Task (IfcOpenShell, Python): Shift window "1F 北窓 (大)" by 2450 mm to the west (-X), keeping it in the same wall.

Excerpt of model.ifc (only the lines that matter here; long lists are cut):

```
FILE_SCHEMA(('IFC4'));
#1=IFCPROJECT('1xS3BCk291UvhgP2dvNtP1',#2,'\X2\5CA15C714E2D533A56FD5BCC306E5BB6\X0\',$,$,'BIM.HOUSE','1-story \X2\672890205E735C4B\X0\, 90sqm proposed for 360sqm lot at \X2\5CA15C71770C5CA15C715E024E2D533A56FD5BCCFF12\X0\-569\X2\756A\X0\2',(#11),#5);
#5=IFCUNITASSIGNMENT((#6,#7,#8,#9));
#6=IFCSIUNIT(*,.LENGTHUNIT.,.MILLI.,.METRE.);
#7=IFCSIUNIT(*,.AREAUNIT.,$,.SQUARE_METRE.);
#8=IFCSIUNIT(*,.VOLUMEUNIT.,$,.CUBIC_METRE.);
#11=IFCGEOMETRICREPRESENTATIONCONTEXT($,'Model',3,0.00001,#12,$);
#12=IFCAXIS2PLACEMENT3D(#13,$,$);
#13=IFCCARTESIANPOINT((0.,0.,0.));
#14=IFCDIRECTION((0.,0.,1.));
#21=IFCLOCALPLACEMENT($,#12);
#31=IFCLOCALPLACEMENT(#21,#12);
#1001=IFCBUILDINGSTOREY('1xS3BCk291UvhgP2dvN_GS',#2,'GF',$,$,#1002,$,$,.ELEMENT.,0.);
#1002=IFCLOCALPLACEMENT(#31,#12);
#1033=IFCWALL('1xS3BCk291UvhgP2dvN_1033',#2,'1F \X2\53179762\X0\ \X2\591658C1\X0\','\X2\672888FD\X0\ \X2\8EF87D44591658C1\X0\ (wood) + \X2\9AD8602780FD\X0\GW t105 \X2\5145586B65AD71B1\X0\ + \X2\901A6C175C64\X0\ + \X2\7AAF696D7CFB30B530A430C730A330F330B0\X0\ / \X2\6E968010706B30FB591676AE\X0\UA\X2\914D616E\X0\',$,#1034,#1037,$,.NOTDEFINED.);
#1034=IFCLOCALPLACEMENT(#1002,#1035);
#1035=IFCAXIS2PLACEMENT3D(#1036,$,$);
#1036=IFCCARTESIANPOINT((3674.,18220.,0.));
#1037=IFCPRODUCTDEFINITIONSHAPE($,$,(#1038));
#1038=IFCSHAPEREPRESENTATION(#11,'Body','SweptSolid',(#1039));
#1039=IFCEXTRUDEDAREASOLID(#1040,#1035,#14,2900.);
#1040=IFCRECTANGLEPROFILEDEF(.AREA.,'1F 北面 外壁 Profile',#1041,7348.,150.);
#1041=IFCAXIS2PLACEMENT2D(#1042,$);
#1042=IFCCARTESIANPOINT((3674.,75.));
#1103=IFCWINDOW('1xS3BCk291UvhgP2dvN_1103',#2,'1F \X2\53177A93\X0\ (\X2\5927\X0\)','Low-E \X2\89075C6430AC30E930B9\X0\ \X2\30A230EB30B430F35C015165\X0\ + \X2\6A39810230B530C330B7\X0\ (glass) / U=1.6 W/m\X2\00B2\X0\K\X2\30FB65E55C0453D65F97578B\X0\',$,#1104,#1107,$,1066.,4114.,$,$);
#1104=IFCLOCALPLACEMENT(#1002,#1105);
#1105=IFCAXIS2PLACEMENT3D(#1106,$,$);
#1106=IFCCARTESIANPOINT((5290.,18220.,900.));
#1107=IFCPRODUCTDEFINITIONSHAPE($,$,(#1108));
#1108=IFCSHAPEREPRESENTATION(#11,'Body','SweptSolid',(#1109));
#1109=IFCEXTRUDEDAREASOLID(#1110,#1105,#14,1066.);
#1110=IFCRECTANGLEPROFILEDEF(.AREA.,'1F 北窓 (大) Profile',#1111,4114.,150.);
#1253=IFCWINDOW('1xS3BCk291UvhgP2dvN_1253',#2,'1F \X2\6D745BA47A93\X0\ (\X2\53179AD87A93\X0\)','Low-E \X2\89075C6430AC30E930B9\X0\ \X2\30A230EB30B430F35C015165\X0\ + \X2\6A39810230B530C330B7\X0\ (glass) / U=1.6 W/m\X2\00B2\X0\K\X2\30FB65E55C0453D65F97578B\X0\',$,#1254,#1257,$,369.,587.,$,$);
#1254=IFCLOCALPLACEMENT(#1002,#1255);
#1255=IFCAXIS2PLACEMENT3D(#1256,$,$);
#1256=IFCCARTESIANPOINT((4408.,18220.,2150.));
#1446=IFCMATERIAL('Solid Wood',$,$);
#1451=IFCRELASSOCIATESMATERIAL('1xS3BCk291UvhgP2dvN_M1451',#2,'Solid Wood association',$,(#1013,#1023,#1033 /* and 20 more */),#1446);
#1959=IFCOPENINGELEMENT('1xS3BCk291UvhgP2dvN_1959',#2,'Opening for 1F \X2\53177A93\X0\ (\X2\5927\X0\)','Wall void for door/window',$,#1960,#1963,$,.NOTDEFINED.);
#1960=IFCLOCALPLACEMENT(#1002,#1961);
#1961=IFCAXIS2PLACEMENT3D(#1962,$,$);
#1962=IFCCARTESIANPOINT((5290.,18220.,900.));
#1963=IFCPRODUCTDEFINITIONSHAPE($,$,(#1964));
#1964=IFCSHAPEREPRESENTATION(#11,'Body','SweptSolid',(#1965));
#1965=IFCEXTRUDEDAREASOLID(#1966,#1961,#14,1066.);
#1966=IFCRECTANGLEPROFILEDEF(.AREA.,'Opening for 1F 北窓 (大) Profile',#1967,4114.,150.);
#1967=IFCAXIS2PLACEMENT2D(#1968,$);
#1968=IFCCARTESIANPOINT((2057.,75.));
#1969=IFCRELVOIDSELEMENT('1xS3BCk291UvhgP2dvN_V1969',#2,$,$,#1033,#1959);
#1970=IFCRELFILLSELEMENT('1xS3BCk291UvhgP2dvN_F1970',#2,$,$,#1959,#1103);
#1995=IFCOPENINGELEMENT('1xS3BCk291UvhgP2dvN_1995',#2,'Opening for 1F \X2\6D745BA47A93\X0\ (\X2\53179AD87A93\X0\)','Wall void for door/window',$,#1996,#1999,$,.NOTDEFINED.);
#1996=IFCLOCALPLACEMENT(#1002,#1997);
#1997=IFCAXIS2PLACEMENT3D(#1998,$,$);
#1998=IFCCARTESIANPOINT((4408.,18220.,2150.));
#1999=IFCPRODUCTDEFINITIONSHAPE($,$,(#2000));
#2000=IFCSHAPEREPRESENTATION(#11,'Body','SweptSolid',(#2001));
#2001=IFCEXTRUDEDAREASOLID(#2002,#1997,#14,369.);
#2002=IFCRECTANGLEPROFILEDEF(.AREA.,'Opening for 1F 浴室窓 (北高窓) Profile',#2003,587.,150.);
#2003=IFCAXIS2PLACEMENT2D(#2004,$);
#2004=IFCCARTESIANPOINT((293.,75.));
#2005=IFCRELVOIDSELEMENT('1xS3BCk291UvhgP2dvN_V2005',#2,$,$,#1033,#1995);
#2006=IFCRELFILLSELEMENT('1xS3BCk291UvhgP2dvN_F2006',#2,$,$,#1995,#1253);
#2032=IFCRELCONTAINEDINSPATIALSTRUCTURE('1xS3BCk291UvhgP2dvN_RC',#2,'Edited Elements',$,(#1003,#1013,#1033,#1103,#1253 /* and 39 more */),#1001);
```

```python
import ifcopenshell
import ifcopenshell.api.geometry
import ifcopenshell.util.placement
import ifcopenshell.util.unit

model = ifcopenshell.open("model.ifc")
unit_scale = ifcopenshell.util.unit.calculate_unit_scale(model)

window = model.by_guid("1xS3BCk291UvhgP2dvN_1103")
opening = window.FillsVoids[0].RelatingOpeningElement
wall = opening.VoidsElements[0].RelatingBuildingElement

wall_matrix = ifcopenshell.util.placement.get_local_placement(wall.ObjectPlacement)
shift = wall_matrix[:3, 0] * -2.45 / unit_scale
before = ifcopenshell.util.placement.get_local_placement(window.ObjectPlacement)[:3, 3].copy()

# The window is not placed relative to its opening, so move both.
for product in (opening, window):
    matrix = ifcopenshell.util.placement.get_local_placement(product.ObjectPlacement)
    matrix[:3, 3] += shift
    ifcopenshell.api.geometry.edit_object_placement(model, product=product, matrix=matrix, is_si=False)

after = ifcopenshell.util.placement.get_local_placement(window.ObjectPlacement)[:3, 3]
print("window moved by", (after - before).round(3) + 0.0)

model.write("model_updated.ifc")
```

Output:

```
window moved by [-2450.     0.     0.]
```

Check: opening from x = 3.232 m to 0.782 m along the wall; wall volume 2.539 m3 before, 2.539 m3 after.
